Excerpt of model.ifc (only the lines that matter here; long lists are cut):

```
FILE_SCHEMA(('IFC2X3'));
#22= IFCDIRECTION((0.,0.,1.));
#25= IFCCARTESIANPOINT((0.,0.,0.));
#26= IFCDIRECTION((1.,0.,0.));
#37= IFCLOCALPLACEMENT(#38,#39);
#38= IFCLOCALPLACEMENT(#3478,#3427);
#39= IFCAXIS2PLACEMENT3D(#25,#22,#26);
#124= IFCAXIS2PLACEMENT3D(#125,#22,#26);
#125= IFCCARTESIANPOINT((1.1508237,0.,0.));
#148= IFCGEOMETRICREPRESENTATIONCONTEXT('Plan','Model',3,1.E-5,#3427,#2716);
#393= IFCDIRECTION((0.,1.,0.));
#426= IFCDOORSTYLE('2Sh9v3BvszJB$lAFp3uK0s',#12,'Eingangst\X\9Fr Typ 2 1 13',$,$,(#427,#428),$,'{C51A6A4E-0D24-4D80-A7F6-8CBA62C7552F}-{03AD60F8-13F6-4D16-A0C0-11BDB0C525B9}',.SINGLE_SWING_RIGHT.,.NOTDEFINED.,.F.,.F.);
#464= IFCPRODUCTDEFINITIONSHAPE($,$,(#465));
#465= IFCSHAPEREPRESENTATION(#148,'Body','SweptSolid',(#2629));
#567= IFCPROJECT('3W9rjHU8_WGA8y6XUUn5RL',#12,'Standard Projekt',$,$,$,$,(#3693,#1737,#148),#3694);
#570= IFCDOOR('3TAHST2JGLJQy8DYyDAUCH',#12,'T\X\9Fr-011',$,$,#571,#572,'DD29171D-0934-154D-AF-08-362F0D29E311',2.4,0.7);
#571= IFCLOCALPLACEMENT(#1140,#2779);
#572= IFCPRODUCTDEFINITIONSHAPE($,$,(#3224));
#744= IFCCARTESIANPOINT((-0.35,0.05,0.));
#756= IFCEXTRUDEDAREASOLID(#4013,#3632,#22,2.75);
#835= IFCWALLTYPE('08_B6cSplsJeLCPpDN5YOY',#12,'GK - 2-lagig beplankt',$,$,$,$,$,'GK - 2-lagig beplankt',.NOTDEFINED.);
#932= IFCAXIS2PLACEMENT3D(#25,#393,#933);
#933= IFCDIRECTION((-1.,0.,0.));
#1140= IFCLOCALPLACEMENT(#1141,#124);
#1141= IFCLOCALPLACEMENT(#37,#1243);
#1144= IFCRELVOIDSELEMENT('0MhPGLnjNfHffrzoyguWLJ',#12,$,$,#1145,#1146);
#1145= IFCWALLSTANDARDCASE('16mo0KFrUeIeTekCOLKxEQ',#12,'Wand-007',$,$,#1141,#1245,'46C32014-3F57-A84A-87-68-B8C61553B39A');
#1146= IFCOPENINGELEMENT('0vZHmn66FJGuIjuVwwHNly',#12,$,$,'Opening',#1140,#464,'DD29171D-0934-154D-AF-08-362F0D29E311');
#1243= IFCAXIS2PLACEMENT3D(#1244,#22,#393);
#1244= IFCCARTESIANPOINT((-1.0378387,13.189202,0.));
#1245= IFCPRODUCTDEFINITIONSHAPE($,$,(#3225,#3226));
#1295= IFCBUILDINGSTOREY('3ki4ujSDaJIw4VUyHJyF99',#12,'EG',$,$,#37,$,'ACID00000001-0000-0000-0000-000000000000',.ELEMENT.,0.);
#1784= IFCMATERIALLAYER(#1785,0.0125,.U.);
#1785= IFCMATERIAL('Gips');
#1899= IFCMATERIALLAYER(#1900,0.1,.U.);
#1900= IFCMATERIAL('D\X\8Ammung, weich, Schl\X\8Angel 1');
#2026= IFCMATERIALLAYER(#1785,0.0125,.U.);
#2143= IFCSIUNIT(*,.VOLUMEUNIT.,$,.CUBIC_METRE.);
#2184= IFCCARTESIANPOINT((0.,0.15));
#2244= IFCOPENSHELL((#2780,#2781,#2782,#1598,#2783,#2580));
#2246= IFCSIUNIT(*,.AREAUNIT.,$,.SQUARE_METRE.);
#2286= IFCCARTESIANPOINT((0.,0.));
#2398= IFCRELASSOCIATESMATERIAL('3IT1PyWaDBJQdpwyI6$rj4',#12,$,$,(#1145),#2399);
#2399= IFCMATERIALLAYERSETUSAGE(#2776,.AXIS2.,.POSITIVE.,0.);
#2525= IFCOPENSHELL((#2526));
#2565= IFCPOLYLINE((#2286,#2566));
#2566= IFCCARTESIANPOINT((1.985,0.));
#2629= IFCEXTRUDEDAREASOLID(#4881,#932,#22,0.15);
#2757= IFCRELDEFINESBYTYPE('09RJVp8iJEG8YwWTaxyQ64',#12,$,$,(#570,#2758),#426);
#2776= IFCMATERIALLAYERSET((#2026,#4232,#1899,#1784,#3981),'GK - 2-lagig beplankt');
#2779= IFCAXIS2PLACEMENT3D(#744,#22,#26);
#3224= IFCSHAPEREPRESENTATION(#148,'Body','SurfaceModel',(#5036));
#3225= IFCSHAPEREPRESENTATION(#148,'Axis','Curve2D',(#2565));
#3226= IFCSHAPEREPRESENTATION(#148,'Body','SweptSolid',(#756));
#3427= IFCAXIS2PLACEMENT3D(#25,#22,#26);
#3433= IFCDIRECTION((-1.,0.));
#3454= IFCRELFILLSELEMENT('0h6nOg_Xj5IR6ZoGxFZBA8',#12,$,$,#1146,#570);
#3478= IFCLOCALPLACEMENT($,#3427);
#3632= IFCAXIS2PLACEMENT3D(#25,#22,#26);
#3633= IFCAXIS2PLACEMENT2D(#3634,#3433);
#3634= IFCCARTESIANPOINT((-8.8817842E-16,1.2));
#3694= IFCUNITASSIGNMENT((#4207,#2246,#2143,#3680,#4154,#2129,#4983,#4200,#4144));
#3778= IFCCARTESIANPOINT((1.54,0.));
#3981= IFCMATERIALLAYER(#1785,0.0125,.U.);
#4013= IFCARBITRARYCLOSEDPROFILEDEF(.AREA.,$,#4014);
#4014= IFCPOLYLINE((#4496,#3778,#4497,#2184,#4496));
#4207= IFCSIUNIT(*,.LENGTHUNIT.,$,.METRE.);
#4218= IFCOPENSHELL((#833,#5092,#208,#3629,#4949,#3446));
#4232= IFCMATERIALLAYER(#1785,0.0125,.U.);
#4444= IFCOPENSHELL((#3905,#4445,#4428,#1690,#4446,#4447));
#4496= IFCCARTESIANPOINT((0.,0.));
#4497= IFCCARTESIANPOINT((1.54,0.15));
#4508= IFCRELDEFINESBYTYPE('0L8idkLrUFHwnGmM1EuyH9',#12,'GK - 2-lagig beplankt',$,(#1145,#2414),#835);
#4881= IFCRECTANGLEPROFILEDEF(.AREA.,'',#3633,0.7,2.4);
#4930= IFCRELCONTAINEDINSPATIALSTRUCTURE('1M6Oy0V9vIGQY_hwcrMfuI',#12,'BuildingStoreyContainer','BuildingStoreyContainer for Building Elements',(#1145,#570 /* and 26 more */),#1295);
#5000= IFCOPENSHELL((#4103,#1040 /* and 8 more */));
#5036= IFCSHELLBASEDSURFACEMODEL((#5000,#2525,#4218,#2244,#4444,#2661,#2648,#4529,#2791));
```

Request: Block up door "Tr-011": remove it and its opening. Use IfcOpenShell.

```python
import ifcopenshell
import ifcopenshell.api.feature
import ifcopenshell.api.root
import ifcopenshell.geom
import ifcopenshell.util.shape

model = ifcopenshell.open("model.ifc")
settings = ifcopenshell.geom.settings()


def volume(element):
    """Net volume in cubic metres, openings subtracted."""
    shape = ifcopenshell.geom.create_shape(settings, element)
    return ifcopenshell.util.shape.get_volume(shape.geometry)


door = model.by_guid("3TAHST2JGLJQy8DYyDAUCH")
opening = door.FillsVoids[0].RelatingOpeningElement
wall = opening.VoidsElements[0].RelatingBuildingElement
before = volume(wall)

ifcopenshell.api.root.remove_product(model, product=door)
ifcopenshell.api.feature.remove_feature(model, feature=opening)

after = volume(wall)

print(f"wall volume {before:.3f} -> {after:.3f} m3")

model.write("model_v2.ifc")
```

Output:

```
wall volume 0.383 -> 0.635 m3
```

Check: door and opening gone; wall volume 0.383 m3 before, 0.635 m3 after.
